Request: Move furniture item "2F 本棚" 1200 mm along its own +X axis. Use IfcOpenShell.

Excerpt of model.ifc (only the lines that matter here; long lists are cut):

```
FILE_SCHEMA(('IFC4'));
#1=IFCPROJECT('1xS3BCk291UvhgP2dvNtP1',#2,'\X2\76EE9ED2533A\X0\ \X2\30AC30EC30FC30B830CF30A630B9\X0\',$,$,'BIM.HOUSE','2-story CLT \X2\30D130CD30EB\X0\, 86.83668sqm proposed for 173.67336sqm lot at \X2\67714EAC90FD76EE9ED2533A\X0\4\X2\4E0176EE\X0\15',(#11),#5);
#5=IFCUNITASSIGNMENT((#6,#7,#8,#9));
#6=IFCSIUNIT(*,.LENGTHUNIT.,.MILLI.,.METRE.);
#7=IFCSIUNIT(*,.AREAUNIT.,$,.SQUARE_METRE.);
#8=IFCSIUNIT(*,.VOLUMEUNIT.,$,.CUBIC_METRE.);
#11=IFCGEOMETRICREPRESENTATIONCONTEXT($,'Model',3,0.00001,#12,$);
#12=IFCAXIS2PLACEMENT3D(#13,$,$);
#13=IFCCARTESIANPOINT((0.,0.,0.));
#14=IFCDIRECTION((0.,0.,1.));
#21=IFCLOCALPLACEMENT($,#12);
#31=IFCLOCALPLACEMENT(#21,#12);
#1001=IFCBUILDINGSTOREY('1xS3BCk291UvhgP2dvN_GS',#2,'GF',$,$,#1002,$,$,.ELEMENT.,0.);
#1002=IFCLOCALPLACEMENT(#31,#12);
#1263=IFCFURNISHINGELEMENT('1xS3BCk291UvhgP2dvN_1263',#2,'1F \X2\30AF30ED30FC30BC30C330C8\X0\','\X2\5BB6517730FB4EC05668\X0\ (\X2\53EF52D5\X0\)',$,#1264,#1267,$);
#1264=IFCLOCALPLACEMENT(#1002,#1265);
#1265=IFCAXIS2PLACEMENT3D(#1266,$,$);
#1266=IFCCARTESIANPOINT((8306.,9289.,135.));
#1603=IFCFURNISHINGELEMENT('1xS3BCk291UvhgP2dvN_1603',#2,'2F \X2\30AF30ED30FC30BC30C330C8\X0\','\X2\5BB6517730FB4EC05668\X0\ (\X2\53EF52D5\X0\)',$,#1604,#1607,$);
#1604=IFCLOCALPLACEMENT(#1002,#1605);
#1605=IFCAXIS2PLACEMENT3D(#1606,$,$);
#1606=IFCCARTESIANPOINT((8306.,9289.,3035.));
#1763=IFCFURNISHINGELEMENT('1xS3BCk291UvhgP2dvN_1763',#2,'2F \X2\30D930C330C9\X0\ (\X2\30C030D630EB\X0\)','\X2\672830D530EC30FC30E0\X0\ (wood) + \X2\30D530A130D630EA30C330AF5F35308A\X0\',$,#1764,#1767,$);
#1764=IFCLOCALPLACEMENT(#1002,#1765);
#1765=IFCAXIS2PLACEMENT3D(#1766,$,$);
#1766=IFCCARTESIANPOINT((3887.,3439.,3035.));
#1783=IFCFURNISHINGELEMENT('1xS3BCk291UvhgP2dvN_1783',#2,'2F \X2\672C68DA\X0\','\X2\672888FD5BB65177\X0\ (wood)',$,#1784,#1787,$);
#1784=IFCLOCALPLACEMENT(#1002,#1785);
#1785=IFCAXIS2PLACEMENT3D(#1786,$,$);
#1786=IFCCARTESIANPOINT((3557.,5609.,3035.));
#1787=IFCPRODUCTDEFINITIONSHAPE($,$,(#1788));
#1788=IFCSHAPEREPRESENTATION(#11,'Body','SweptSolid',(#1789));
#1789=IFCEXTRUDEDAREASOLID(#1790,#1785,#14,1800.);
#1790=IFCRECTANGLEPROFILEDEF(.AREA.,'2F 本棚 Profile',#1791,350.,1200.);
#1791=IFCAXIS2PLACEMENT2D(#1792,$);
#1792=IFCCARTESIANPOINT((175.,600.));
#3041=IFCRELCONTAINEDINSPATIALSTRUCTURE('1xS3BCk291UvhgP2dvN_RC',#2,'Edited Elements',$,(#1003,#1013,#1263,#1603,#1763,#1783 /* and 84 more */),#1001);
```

```python
import ifcopenshell
import ifcopenshell.api.geometry
import ifcopenshell.util.placement
import ifcopenshell.util.unit

model = ifcopenshell.open("model.ifc")
unit_scale = ifcopenshell.util.unit.calculate_unit_scale(model)

item = model.by_guid("1xS3BCk291UvhgP2dvN_1783")
matrix = ifcopenshell.util.placement.get_local_placement(item.ObjectPlacement)
matrix[:3, 3] += matrix[:3, 0] * 1.2 / unit_scale
ifcopenshell.api.geometry.edit_object_placement(model, product=item, matrix=matrix, is_si=False)

print(ifcopenshell.util.placement.get_local_placement(item.ObjectPlacement).round(3) + 0.0)

model.write("model_rev.ifc")
```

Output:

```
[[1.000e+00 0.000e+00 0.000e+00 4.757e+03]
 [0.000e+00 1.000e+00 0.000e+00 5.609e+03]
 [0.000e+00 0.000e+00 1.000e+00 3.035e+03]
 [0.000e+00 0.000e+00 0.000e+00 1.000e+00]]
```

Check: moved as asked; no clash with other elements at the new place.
